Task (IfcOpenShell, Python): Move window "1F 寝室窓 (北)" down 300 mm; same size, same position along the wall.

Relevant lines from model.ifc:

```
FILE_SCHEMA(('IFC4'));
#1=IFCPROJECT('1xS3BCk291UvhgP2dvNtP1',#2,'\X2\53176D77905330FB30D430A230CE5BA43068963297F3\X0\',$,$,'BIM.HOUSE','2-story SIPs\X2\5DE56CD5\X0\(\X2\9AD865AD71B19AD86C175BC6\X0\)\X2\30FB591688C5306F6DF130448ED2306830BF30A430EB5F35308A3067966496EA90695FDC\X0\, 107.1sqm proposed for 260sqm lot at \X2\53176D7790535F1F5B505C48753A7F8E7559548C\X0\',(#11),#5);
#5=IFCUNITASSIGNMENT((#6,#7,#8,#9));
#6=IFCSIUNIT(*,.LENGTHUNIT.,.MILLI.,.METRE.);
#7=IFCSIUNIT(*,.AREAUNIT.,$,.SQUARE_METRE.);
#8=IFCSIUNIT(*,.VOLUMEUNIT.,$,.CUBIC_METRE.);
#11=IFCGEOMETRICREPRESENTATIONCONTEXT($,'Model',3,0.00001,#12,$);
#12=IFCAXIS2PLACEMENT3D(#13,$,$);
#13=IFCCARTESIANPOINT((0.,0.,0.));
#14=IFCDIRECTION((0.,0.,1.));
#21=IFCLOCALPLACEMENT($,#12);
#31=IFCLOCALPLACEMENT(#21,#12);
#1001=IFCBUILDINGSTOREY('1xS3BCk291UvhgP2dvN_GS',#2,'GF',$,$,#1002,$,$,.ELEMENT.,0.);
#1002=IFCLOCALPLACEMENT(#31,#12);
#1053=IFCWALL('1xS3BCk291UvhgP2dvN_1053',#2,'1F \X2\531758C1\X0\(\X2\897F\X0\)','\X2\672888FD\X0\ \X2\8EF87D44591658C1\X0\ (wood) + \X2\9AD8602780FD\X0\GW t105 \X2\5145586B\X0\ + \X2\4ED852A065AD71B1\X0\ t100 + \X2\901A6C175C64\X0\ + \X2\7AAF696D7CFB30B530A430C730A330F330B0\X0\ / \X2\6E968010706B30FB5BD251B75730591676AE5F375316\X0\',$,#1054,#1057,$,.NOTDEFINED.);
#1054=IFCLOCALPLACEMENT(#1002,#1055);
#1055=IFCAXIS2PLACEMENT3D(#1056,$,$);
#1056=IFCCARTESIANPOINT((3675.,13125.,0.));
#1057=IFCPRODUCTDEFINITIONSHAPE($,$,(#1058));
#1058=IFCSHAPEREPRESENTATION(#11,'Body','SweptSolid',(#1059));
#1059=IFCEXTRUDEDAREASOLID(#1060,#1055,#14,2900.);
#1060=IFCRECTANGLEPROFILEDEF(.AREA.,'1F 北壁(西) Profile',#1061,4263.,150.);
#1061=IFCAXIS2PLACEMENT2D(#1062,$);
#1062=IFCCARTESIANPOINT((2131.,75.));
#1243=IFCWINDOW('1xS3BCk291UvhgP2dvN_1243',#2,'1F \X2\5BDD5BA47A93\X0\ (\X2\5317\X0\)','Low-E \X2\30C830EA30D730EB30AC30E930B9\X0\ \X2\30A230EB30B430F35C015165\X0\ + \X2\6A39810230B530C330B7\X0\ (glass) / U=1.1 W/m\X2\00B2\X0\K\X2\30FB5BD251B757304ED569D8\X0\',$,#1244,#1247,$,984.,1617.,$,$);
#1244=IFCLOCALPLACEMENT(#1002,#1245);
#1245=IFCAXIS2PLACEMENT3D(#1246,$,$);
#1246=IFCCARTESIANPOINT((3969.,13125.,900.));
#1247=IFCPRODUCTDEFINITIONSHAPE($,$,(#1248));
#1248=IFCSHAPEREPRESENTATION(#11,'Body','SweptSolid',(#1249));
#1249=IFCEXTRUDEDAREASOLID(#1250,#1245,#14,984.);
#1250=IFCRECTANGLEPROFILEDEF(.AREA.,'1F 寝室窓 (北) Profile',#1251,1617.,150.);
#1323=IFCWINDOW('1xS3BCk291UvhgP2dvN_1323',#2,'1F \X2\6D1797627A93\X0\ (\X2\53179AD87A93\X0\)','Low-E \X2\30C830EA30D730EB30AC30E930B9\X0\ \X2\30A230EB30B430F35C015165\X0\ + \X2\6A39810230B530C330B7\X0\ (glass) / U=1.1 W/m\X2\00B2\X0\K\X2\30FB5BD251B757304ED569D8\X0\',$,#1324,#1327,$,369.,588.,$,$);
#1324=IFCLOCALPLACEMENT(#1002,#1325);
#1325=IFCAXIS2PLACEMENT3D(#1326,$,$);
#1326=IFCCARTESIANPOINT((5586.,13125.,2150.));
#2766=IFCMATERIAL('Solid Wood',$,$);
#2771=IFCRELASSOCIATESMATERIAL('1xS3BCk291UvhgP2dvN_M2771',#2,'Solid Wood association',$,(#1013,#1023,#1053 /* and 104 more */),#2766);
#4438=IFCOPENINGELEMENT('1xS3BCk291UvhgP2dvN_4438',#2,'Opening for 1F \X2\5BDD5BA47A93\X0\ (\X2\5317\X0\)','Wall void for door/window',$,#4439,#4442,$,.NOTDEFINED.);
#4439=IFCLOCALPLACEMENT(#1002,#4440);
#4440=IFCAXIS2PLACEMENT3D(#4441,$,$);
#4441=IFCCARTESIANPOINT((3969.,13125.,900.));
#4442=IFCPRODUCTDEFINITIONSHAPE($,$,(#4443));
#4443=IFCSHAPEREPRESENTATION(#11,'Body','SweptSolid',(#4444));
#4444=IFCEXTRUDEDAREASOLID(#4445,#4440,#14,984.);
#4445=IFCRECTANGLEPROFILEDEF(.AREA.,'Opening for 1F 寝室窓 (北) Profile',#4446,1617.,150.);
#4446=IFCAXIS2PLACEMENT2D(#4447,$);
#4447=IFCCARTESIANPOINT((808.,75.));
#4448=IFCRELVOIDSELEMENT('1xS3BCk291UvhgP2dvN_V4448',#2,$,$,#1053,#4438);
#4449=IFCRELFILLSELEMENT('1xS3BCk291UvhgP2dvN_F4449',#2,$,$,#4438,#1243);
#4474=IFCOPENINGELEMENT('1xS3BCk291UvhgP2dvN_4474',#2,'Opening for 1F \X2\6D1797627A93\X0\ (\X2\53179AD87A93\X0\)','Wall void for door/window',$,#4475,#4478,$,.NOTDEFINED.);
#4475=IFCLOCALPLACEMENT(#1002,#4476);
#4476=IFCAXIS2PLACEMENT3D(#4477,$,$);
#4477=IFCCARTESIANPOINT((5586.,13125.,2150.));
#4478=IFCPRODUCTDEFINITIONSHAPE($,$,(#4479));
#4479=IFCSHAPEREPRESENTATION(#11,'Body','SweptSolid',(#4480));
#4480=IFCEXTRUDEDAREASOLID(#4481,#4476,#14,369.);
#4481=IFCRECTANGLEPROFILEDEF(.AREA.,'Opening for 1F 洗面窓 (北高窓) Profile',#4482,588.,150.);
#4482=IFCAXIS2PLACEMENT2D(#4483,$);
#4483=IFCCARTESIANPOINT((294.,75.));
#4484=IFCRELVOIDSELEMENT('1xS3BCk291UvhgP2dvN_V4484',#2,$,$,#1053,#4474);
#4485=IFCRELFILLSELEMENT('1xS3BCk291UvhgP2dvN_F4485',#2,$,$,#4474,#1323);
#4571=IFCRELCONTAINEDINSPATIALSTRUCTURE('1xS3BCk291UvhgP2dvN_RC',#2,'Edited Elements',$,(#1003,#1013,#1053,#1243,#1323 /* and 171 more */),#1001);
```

```python
import numpy as np
import ifcopenshell
import ifcopenshell.api.geometry
import ifcopenshell.util.placement
import ifcopenshell.util.unit

model = ifcopenshell.open("model.ifc")
unit_scale = ifcopenshell.util.unit.calculate_unit_scale(model)

window = model.by_id(1243)
opening = window.FillsVoids[0].RelatingOpeningElement
dz = -0.3 / unit_scale

shift = np.array([0.0, 0.0, dz])
# The window is not placed relative to its opening, so move both.
for product in (opening, window):
    matrix = ifcopenshell.util.placement.get_local_placement(product.ObjectPlacement)
    matrix[:3, 3] += shift
    ifcopenshell.api.geometry.edit_object_placement(model, product=product, matrix=matrix, is_si=False)

print(f"moved by {dz * unit_scale:+.3f} m")

model.write("model-out.ifc")
```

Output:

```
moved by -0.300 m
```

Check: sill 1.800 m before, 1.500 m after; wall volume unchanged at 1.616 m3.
